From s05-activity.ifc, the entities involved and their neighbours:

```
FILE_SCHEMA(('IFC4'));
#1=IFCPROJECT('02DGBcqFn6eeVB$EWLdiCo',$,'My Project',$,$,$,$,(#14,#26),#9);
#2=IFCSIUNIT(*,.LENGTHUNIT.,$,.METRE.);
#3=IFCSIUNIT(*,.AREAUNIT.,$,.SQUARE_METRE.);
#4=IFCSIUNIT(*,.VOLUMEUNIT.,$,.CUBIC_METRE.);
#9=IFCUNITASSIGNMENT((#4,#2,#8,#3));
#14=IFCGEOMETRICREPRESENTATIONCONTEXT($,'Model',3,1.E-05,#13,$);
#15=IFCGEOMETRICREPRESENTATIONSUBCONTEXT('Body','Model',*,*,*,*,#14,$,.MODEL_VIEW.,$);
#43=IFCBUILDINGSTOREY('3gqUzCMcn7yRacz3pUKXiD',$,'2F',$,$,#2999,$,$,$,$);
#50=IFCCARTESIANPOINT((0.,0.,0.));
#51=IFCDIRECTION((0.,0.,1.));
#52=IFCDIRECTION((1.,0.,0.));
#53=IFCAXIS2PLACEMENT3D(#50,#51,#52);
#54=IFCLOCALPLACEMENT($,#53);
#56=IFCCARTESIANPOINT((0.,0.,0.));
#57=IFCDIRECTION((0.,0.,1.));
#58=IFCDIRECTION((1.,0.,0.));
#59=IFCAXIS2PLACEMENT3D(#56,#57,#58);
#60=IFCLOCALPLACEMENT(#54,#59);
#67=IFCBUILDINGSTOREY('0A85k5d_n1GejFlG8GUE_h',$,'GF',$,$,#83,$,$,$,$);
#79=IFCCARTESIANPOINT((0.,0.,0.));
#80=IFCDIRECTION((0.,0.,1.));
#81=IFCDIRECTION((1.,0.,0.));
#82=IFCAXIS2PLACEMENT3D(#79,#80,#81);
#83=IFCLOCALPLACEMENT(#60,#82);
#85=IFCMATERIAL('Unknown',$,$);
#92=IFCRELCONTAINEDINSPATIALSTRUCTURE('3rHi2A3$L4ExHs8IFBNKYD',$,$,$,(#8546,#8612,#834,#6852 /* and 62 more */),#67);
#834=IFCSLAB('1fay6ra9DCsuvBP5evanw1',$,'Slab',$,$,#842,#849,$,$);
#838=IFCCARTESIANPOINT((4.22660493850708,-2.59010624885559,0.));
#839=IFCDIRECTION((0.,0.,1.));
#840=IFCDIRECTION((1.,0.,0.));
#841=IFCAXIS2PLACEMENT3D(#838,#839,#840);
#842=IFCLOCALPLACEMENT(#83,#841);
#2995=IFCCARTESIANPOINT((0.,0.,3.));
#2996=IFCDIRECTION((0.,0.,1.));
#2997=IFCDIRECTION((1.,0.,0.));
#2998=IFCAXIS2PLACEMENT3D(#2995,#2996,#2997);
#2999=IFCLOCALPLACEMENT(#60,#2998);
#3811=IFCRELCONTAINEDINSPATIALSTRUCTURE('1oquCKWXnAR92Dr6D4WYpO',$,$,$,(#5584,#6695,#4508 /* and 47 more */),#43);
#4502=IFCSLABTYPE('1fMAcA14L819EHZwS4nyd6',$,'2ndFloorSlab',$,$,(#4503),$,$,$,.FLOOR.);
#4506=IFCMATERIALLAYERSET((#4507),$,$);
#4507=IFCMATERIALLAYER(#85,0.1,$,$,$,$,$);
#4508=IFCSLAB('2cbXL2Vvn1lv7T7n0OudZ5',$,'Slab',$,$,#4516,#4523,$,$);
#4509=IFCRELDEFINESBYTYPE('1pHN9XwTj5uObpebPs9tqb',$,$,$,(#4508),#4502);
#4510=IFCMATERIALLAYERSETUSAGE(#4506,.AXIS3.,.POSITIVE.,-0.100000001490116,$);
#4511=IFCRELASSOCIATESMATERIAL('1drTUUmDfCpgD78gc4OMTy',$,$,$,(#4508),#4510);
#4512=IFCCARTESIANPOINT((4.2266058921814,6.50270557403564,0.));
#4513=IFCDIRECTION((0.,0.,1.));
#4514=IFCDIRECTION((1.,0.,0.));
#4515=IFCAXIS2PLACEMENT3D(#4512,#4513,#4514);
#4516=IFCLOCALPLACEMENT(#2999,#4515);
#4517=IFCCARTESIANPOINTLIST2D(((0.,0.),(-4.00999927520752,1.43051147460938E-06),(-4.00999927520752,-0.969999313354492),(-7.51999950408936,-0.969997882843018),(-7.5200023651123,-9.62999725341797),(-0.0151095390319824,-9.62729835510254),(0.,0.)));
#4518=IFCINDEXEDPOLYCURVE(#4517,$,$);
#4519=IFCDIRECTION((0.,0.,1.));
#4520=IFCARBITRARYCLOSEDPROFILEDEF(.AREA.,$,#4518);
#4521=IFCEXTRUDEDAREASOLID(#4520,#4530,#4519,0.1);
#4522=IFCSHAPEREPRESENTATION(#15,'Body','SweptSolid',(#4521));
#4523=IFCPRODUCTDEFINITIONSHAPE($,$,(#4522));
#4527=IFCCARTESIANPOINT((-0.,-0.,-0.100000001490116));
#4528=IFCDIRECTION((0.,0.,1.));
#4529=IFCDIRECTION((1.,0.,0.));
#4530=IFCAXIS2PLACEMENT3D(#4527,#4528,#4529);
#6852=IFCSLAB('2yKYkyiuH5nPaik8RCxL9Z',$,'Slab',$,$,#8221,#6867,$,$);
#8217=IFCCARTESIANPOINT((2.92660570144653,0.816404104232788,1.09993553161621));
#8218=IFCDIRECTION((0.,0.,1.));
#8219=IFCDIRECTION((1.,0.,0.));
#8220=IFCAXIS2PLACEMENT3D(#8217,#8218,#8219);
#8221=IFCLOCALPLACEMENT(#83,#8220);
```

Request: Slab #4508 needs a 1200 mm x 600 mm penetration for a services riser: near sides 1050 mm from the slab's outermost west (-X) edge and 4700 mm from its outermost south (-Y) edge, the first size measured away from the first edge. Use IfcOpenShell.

```python
import numpy as np
import ifcopenshell
import ifcopenshell.api.feature
import ifcopenshell.api.geometry
import ifcopenshell.api.root
import ifcopenshell.geom
import ifcopenshell.util.placement
import ifcopenshell.util.representation
import ifcopenshell.util.shape
import ifcopenshell.util.unit

model = ifcopenshell.open("s05-activity.ifc")
unit_scale = ifcopenshell.util.unit.calculate_unit_scale(model)
settings = ifcopenshell.geom.settings()


def volume(element):
    """Net volume in cubic metres, openings subtracted."""
    shape = ifcopenshell.geom.create_shape(settings, element)
    return ifcopenshell.util.shape.get_volume(shape.geometry)


slab = model.by_id(4508)
before = volume(slab)

# Extent in the slab's own axes, in metres. The edges named are its -X and -Y sides.
slab_shape = ifcopenshell.geom.create_shape(settings, slab)
vertices = ifcopenshell.util.shape.get_vertices(slab_shape.geometry)
x_min, y_min, bottom = vertices.min(axis=0)
top = vertices[:, 2].max()

opening = ifcopenshell.api.root.create_entity(model, ifc_class="IfcOpeningElement", name="Services riser opening", predefined_type="OPENING")
context = ifcopenshell.util.representation.get_context(model, "Model", "Body", "MODEL_VIEW")
width, depth = 1.2, 0.6
outline = [(0.0, 0.0), (width, 0.0), (width, depth), (0.0, depth), (0.0, 0.0)]
# Overshoot both faces by 50 mm so the cut is clean.
shape = ifcopenshell.api.geometry.add_slab_representation(
    model, context=context, depth=top - bottom + 0.1, polyline=outline
)
ifcopenshell.api.geometry.assign_representation(model, product=opening, representation=shape)

matrix = ifcopenshell.util.placement.get_local_placement(slab.ObjectPlacement)
matrix[:, 3] = matrix @ np.append(np.array([x_min + 1.05, y_min + 4.7, bottom - 0.05]) / unit_scale, 1.0)
ifcopenshell.api.geometry.edit_object_placement(model, product=opening, matrix=matrix, is_si=False)
ifcopenshell.api.feature.add_feature(model, feature=opening, element=slab)

after = volume(slab)

print(f"slab volume {before:.3f} -> {after:.3f} m3")

model.write("s05-activity_updated.ifc")
```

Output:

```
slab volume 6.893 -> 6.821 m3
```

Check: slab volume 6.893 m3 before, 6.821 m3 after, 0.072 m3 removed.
